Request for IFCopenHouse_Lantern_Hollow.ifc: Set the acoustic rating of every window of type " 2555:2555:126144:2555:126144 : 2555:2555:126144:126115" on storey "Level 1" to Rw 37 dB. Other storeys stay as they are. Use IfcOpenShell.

First a look at what the model holds.

```python
import ifcopenshell
import ifcopenshell.util.element

model = ifcopenshell.open("IFCopenHouse_Lantern_Hollow.ifc")
print(model.schema)
storey = next(s for s in model.by_type("IfcBuildingStorey") if s.Name == "Level 1")
windows = [e for e in ifcopenshell.util.element.get_decomposition(storey) if e.is_a("IfcWindow")]
seen = {}
for e in windows:
    element_type = ifcopenshell.util.element.get_type(e)
    key = (element_type.Name if element_type != e and element_type else None, ifcopenshell.util.element.get_pset(e, "Pset_WindowCommon", "AcousticRating"))
    seen[key] = seen.get(key, 0) + 1
for (name, value), count in sorted(seen.items(), key=str):
    print(count, "x", name, "|", value)
```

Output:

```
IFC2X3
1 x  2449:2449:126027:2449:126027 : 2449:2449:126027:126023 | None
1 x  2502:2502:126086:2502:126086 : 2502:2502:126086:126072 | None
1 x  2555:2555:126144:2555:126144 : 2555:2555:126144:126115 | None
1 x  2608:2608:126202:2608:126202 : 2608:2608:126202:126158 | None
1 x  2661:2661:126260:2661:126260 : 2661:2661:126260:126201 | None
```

```python
import ifcopenshell
import ifcopenshell.api.pset
import ifcopenshell.util.element

model = ifcopenshell.open("IFCopenHouse_Lantern_Hollow.ifc")

storey = next(s for s in model.by_type("IfcBuildingStorey") if s.Name == "Level 1")
windows = [e for e in ifcopenshell.util.element.get_decomposition(storey) if e.is_a("IfcWindow")]

count = 0
for e in windows:
    element_type = ifcopenshell.util.element.get_type(e)
    if element_type in (None, e) or element_type.Name != " 2555:2555:126144:2555:126144 : 2555:2555:126144:126115":
        continue
    # add_pset returns the element's existing set when there is one.
    pset = ifcopenshell.api.pset.add_pset(model, product=e, name="Pset_WindowCommon")
    ifcopenshell.api.pset.edit_pset(model, pset=pset, properties={"AcousticRating": "Rw 37 dB"})
    count += 1

print(count, "windows updated")

model.write("IFCopenHouse_Lantern_Hollow_v2.ifc")
```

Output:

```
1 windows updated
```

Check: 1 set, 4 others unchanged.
